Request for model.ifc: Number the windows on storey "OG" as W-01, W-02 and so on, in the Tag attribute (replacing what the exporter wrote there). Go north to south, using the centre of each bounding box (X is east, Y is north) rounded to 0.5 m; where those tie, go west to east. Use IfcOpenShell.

First a look at what the model holds.

```python
import ifcopenshell
import ifcopenshell.util.element
import ifcopenshell.util.placement

model = ifcopenshell.open("model.ifc")
print(model.schema)
storey = next(s for s in model.by_type("IfcBuildingStorey") if s.Name == "OG")
windows = [e for e in ifcopenshell.util.element.get_decomposition(storey) if e.is_a("IfcWindow")]
for e in sorted(windows, key=lambda e: e.id()):
    origin = ifcopenshell.util.placement.get_local_placement(e.ObjectPlacement)[:3, 3]
    print(e.id(), e.Tag, e.Name, origin.round(2) + 0.0, sep=" | ")
```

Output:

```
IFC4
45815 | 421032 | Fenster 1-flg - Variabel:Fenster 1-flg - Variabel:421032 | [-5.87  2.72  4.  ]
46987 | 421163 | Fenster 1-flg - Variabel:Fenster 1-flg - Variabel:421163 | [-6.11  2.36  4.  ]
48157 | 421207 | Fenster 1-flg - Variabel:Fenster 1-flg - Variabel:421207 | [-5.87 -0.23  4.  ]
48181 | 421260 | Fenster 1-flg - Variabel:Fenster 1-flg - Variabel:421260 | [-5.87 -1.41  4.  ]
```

```python
import ifcopenshell
import ifcopenshell.geom
import ifcopenshell.util.element
import ifcopenshell.util.shape

model = ifcopenshell.open("model.ifc")
settings = ifcopenshell.geom.settings()
settings.set("use-world-coords", True)


def centre(element):
    shape = ifcopenshell.geom.create_shape(settings, element)
    return ifcopenshell.util.shape.get_bbox_centroid(shape.geometry)


storey = next(s for s in model.by_type("IfcBuildingStorey") if s.Name == "OG")
windows = [e for e in ifcopenshell.util.element.get_decomposition(storey) if e.is_a("IfcWindow")]

# Insertion points can sit at a corner or the storey origin, so sort by the geometry (in metres).
centres = {e: centre(e) for e in windows}
windows.sort(key=lambda e: (-round(centres[e][1] / 0.5), centres[e][0]))

for i, e in enumerate(windows, start=1):
    number = f"W-{i:02d}"
    e.Tag = number
    print(e.id(), number)

model.write("model_rev.ifc")
```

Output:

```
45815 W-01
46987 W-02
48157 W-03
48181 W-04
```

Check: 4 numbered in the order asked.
